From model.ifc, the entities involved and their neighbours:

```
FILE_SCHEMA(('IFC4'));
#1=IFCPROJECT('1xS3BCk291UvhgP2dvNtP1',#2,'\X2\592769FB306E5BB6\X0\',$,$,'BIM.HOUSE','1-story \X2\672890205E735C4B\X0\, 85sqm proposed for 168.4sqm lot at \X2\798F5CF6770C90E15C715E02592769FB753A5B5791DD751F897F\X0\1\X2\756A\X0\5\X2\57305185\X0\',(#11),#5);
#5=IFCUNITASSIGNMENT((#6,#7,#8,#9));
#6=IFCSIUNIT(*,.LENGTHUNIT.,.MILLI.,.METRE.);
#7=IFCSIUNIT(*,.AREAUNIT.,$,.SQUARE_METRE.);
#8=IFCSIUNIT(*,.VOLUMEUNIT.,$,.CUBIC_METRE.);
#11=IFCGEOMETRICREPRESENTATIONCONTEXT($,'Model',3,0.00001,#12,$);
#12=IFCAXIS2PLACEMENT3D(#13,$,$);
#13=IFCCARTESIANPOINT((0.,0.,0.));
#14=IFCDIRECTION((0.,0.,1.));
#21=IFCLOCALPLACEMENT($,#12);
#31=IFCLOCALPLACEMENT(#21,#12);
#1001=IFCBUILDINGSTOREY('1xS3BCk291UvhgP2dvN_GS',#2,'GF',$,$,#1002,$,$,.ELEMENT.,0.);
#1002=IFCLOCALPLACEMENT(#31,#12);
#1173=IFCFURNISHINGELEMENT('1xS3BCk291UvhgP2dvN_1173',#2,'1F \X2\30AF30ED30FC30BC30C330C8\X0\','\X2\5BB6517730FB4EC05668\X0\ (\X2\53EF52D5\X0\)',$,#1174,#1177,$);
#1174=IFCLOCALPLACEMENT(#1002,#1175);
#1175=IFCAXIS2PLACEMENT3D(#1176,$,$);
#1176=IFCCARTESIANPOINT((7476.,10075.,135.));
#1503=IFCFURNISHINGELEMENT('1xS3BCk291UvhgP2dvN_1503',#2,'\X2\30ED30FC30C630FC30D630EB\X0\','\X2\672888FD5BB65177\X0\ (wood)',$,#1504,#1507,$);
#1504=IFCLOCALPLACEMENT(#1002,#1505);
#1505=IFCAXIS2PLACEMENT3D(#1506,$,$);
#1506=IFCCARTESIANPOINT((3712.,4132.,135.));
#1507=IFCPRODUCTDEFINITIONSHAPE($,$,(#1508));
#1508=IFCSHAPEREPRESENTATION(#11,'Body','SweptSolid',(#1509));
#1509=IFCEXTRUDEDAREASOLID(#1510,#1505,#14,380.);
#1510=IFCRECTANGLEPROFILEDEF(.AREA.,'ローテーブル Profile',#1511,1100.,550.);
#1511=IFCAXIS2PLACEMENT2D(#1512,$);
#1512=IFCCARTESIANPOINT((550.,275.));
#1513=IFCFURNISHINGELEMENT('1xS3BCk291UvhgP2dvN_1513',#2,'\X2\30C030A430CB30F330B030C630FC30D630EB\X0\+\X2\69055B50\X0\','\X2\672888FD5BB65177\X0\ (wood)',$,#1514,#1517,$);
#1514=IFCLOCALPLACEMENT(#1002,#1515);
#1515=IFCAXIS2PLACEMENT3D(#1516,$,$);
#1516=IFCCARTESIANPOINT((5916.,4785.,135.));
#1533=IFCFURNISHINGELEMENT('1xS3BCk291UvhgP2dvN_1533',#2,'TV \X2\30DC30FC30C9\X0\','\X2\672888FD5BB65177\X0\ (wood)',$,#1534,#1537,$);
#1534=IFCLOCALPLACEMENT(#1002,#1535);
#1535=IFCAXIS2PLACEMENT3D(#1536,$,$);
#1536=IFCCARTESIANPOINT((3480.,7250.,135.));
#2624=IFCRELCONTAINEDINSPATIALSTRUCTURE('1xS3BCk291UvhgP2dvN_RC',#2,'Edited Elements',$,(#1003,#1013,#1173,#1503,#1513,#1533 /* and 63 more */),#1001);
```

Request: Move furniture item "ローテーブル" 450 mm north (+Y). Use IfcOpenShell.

```python
import ifcopenshell
import ifcopenshell.api.geometry
import ifcopenshell.util.placement
import ifcopenshell.util.unit

model = ifcopenshell.open("model.ifc")
unit_scale = ifcopenshell.util.unit.calculate_unit_scale(model)

item = model.by_guid("1xS3BCk291UvhgP2dvN_1503")
matrix = ifcopenshell.util.placement.get_local_placement(item.ObjectPlacement)
matrix[1, 3] += 0.45 / unit_scale
ifcopenshell.api.geometry.edit_object_placement(model, product=item, matrix=matrix, is_si=False)

print(ifcopenshell.util.placement.get_local_placement(item.ObjectPlacement).round(3) + 0.0)

model.write("model_updated.ifc")
```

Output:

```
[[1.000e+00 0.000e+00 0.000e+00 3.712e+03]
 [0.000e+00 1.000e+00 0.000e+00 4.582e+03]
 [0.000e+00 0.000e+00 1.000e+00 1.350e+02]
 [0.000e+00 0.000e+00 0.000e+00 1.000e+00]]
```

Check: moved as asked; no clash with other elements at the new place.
